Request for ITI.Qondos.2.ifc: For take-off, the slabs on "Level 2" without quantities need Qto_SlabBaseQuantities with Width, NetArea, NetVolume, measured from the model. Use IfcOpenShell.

First a look at what the model holds.

```python
import ifcopenshell
import ifcopenshell.util.element
import ifcopenshell.util.unit

model = ifcopenshell.open("ITI.Qondos.2.ifc")
print(model.schema)
for unit_type in ("LENGTHUNIT", "AREAUNIT", "VOLUMEUNIT"):
    print(unit_type, ifcopenshell.util.unit.calculate_unit_scale(model, unit_type))
storey = next(s for s in model.by_type("IfcBuildingStorey") if s.Name == "Level 2")
slabs = [e for e in ifcopenshell.util.element.get_decomposition(storey) if e.is_a("IfcSlab")]
for e in sorted(slabs, key=lambda e: e.id()):
    print(e.id(), e.is_a(), e.Name, list(ifcopenshell.util.element.get_psets(e, qtos_only=True)), sep=" | ")
```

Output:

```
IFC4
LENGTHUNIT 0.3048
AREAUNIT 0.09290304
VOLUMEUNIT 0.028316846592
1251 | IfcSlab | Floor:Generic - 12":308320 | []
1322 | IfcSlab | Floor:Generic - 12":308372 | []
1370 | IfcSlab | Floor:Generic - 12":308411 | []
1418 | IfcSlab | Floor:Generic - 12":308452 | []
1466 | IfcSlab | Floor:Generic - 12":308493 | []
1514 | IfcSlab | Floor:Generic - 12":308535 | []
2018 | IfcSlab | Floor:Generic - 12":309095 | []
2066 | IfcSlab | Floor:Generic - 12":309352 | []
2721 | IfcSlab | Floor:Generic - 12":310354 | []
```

```python
import ifcopenshell
import ifcopenshell.api.pset
import ifcopenshell.geom
import ifcopenshell.util.element
import ifcopenshell.util.shape
import ifcopenshell.util.unit

model = ifcopenshell.open("ITI.Qondos.2.ifc")
unit_scale = ifcopenshell.util.unit.calculate_unit_scale(model)
area_scale = ifcopenshell.util.unit.calculate_unit_scale(model, "AREAUNIT")
volume_scale = ifcopenshell.util.unit.calculate_unit_scale(model, "VOLUMEUNIT")
settings = ifcopenshell.geom.settings()

storey = next(s for s in model.by_type("IfcBuildingStorey") if s.Name == "Level 2")
slabs = [e for e in ifcopenshell.util.element.get_decomposition(storey) if e.is_a("IfcSlab")]

for e in sorted(slabs, key=lambda e: e.id()):
    if ifcopenshell.util.element.get_psets(e, qtos_only=True, should_inherit=False):
        continue
    # Geometry comes back in metres, in the element's own axes.
    shape = ifcopenshell.geom.create_shape(settings, e)
    values = {
        "Width": ifcopenshell.util.shape.get_z(shape.geometry) / unit_scale,
        "NetArea": ifcopenshell.util.shape.get_footprint_area(shape.geometry) / area_scale,
        "NetVolume": ifcopenshell.util.shape.get_volume(shape.geometry) / volume_scale,
    }
    qto = ifcopenshell.api.pset.add_qto(model, product=e, name="Qto_SlabBaseQuantities")
    ifcopenshell.api.pset.edit_qto(model, qto=qto, properties=values)
    print(e.id(), {k: round(v, 3) for k, v in values.items()})

model.write("ITI.Qondos.2_updated.ifc")
```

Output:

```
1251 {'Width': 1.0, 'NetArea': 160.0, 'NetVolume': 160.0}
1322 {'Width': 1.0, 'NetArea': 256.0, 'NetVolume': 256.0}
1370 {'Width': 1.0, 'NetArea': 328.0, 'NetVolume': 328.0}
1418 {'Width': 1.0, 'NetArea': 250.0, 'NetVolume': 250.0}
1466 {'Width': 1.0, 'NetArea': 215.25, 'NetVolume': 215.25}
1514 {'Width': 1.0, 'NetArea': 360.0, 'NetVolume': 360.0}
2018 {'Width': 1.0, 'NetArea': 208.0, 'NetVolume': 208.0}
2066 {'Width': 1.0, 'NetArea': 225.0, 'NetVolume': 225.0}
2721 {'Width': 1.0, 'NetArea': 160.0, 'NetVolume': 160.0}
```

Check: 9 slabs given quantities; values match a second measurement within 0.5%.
